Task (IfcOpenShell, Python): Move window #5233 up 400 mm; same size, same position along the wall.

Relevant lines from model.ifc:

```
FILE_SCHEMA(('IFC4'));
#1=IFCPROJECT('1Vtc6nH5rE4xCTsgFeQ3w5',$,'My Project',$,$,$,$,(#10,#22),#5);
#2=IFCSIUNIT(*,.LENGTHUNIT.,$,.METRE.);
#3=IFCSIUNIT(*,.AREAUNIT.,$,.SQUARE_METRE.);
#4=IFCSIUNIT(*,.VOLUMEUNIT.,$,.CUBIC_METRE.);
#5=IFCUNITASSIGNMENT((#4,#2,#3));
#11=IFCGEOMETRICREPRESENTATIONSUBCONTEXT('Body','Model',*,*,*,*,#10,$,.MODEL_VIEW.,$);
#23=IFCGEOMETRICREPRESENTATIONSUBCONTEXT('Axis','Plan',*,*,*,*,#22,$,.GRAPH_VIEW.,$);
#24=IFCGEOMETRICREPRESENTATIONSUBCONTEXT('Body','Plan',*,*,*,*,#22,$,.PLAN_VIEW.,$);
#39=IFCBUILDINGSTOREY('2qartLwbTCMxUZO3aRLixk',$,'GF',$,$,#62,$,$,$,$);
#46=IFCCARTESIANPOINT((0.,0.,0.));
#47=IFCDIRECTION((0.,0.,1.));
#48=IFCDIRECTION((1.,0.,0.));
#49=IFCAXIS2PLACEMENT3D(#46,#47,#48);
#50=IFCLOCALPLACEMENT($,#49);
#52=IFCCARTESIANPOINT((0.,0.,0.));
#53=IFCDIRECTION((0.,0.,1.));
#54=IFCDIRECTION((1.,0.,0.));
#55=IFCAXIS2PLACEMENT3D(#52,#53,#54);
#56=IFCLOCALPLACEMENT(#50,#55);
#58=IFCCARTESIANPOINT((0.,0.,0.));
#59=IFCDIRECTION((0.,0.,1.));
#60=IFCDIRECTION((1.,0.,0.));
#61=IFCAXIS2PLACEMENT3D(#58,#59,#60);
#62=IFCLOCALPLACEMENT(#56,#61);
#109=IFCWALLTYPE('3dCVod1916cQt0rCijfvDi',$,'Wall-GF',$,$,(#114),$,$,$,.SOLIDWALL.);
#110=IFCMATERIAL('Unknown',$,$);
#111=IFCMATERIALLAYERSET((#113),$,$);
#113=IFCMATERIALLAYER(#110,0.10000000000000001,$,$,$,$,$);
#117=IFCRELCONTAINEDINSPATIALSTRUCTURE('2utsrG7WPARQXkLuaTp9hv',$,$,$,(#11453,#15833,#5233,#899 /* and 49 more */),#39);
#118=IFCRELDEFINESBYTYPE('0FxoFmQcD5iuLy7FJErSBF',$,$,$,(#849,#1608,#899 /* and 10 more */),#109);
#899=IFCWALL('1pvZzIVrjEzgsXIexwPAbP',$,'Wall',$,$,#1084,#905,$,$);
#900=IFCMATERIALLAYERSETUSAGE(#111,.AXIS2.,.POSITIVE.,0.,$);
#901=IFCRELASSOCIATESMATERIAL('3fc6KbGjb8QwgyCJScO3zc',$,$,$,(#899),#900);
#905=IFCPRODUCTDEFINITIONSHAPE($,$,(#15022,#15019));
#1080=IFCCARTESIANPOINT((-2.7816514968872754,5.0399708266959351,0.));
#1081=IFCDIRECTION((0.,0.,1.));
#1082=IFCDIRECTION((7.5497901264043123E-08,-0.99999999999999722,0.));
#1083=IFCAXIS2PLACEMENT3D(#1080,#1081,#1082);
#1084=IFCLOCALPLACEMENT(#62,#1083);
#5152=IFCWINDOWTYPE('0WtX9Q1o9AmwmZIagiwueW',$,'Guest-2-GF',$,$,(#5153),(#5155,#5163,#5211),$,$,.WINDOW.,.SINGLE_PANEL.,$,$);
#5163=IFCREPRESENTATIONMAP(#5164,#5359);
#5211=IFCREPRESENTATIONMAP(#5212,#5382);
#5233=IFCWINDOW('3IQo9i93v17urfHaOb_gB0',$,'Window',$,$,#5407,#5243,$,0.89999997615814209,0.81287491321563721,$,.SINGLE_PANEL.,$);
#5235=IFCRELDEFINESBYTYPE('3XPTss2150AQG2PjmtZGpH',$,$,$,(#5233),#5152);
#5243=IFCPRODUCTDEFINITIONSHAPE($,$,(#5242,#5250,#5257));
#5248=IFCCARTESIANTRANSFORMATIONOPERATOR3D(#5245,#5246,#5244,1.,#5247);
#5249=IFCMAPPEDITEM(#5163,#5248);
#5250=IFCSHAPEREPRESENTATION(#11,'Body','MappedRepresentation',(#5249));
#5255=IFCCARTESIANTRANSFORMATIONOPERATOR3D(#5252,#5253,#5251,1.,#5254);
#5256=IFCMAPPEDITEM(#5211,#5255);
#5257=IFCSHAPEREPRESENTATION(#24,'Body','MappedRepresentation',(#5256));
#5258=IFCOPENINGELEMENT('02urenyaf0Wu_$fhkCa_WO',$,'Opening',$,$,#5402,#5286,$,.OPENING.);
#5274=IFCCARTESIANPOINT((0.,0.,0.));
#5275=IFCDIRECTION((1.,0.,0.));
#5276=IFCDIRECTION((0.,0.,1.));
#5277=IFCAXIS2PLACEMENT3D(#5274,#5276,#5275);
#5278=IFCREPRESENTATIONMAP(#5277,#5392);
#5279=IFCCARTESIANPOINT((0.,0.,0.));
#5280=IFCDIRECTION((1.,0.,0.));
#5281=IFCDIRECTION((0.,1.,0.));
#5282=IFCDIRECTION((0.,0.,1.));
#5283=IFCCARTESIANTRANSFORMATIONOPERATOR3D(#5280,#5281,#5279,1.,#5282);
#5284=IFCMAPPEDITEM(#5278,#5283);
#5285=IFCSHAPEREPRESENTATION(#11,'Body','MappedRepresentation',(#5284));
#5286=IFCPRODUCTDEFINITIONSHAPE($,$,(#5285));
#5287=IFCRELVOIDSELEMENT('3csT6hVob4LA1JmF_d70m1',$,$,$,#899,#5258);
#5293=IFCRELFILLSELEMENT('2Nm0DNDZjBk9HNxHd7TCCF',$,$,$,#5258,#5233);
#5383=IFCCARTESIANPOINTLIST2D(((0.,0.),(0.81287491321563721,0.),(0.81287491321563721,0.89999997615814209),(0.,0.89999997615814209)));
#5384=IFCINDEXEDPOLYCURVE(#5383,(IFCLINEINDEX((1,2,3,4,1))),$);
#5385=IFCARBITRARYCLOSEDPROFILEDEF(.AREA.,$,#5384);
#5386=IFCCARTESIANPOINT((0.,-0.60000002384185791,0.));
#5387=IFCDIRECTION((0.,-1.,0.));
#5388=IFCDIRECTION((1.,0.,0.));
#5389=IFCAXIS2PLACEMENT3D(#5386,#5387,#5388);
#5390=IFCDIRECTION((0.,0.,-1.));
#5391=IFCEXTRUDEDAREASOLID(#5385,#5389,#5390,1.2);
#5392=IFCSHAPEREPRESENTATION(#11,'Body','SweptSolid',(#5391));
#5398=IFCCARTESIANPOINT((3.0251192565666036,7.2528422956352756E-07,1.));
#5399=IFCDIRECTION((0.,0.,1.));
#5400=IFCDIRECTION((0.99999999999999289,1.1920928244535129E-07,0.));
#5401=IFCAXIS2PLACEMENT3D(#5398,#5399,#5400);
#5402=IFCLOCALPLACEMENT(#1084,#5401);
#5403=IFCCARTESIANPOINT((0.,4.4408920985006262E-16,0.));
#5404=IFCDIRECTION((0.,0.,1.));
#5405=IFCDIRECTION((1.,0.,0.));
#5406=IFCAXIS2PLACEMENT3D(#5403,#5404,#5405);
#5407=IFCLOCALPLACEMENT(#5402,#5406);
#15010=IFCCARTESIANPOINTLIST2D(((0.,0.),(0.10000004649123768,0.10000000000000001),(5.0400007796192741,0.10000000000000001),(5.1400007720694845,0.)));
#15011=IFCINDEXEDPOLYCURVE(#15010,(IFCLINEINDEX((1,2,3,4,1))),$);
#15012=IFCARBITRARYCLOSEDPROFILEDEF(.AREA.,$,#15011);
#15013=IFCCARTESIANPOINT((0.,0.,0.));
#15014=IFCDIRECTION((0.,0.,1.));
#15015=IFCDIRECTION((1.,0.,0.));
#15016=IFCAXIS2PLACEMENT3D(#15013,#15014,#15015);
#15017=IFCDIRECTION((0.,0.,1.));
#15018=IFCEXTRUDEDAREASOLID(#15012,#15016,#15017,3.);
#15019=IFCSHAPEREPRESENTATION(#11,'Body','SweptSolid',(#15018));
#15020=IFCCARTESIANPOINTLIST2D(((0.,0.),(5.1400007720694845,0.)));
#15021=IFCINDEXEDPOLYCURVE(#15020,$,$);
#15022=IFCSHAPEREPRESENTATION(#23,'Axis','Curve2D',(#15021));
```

```python
import numpy as np
import ifcopenshell
import ifcopenshell.api.geometry
import ifcopenshell.util.placement
import ifcopenshell.util.unit

model = ifcopenshell.open("model.ifc")
unit_scale = ifcopenshell.util.unit.calculate_unit_scale(model)

window = model.by_guid("3IQo9i93v17urfHaOb_gB0")
opening = window.FillsVoids[0].RelatingOpeningElement
dz = 0.4 / unit_scale

shift = np.array([0.0, 0.0, dz])
# The window is placed relative to its opening, so it follows when the opening moves.
matrix = ifcopenshell.util.placement.get_local_placement(opening.ObjectPlacement)
matrix[:3, 3] += shift
ifcopenshell.api.geometry.edit_object_placement(
    model, product=opening, matrix=matrix, is_si=False, should_transform_children=True
)

print(f"moved by {dz * unit_scale:+.3f} m")

model.write("model_v2.ifc")
```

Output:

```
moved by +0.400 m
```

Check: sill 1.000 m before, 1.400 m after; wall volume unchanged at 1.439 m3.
